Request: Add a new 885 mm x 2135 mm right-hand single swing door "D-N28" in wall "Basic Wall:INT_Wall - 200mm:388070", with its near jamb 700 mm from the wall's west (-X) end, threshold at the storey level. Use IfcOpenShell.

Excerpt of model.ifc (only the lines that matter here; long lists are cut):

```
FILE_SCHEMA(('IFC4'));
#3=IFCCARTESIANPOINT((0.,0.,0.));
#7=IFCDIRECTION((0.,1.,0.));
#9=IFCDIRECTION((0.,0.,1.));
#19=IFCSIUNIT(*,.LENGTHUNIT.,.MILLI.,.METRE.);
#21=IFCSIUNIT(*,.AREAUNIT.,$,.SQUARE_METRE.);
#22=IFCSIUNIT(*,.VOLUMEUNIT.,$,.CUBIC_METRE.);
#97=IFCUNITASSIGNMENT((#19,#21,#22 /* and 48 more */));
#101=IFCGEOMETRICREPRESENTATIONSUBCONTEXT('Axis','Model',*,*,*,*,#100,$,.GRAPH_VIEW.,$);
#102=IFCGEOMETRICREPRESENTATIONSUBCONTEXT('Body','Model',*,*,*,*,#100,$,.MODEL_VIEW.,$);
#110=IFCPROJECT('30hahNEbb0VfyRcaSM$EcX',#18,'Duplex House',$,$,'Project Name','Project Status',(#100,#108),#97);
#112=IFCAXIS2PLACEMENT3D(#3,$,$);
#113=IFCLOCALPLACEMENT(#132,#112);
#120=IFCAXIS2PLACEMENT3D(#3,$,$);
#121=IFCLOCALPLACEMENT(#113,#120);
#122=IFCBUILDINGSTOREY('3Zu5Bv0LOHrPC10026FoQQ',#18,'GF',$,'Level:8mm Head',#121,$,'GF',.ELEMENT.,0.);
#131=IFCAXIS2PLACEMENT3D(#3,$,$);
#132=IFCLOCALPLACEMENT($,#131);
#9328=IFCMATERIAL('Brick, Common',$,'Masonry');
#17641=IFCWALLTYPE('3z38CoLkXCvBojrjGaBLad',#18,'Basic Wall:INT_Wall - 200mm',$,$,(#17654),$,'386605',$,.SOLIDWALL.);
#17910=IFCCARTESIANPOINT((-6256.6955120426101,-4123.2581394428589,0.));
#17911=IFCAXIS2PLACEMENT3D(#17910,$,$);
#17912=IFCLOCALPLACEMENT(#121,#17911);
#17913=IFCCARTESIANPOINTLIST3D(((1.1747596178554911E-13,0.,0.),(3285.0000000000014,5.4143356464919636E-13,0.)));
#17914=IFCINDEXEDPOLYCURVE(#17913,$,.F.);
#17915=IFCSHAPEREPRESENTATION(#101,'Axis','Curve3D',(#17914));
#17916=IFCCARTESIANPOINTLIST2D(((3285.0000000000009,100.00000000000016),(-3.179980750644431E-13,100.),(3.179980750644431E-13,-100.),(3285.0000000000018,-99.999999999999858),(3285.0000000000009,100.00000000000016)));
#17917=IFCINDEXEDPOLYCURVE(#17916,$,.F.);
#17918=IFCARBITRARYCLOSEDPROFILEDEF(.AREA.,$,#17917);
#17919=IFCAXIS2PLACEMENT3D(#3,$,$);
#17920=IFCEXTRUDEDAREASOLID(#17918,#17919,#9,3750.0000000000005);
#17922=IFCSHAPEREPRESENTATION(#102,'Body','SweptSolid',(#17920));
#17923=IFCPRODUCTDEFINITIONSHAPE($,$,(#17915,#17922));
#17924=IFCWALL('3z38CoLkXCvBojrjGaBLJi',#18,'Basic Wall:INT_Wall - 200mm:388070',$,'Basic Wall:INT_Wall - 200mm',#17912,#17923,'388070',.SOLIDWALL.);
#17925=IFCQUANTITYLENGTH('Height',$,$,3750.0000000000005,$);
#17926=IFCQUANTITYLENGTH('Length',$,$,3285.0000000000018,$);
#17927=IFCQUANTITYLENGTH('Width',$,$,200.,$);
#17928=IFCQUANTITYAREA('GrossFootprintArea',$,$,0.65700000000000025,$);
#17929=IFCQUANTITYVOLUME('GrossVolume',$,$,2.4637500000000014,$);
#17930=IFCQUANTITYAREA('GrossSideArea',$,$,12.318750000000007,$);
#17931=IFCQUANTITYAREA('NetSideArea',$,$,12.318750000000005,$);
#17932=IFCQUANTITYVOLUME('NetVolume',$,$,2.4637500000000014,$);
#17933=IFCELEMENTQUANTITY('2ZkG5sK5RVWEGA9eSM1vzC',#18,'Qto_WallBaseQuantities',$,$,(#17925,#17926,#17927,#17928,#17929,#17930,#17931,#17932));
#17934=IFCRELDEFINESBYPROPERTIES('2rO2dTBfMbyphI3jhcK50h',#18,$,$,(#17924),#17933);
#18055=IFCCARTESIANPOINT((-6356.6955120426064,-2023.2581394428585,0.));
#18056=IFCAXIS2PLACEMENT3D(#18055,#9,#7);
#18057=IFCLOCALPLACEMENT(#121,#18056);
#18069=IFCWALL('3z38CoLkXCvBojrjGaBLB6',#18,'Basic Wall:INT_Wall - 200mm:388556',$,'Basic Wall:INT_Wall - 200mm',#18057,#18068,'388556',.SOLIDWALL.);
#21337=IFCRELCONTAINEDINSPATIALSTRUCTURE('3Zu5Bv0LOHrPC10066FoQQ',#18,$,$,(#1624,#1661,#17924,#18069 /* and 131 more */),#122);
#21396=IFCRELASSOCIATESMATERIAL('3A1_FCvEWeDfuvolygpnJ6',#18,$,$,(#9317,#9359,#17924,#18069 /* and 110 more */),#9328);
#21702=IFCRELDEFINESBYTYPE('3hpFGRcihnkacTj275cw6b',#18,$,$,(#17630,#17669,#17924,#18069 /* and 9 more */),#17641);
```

```python
import numpy as np
import ifcopenshell
import ifcopenshell.api.feature
import ifcopenshell.api.geometry
import ifcopenshell.api.pset
import ifcopenshell.api.root
import ifcopenshell.api.spatial
import ifcopenshell.geom
import ifcopenshell.util.element
import ifcopenshell.util.placement
import ifcopenshell.util.representation
import ifcopenshell.util.shape
import ifcopenshell.util.unit

model = ifcopenshell.open("model.ifc")
unit_scale = ifcopenshell.util.unit.calculate_unit_scale(model)
area_scale = ifcopenshell.util.unit.calculate_unit_scale(model, "AREAUNIT")
volume_scale = ifcopenshell.util.unit.calculate_unit_scale(model, "VOLUMEUNIT")
settings = ifcopenshell.geom.settings()


def volume(element):
    """Net volume in cubic metres, openings subtracted."""
    shape = ifcopenshell.geom.create_shape(settings, element)
    return ifcopenshell.util.shape.get_volume(shape.geometry)


wall = model.by_guid("3z38CoLkXCvBojrjGaBLJi")
storey = ifcopenshell.util.element.get_container(wall, ifc_class="IfcBuildingStorey")
context = ifcopenshell.util.representation.get_context(model, "Model", "Body", "MODEL_VIEW")
before = volume(wall)

width, height, from_end, sill = 0.885, 2.135, 0.7, 0.0  # metres

# The wall runs along its own X axis, and the end named is its -X end.
wall_shape = ifcopenshell.geom.create_shape(settings, wall)
x, y, z = ifcopenshell.util.shape.get_vertices(wall_shape.geometry).T
start = x.min() + from_end
face, thickness = float(y.min()), float(y.max() - y.min())
wall_matrix = ifcopenshell.util.placement.get_local_placement(wall.ObjectPlacement)
level = ifcopenshell.util.placement.get_local_placement(storey.ObjectPlacement)[2, 3]


def in_wall(x, y):
    """Placement at x, y metres in the wall's axes, at sill height."""
    matrix = wall_matrix.copy()
    matrix[:, 3] = wall_matrix @ np.array([x / unit_scale, y / unit_scale, 0.0, 1.0])
    matrix[2, 3] = level + sill / unit_scale
    return matrix


# Opening: a box that overshoots both wall faces by 50 mm.
opening = ifcopenshell.api.root.create_entity(model, ifc_class="IfcOpeningElement", predefined_type="OPENING")
box = ifcopenshell.api.geometry.add_wall_representation(
    model, context=context, length=width, height=height, thickness=thickness + 0.1
)
ifcopenshell.api.geometry.assign_representation(model, product=opening, representation=box)
ifcopenshell.api.geometry.edit_object_placement(model, product=opening, matrix=in_wall(start, face - 0.05), is_si=False)
ifcopenshell.api.feature.add_feature(model, feature=opening, element=wall)

door = ifcopenshell.api.root.create_entity(model, ifc_class="IfcDoor", name="D-N28", predefined_type="DOOR")
door.OverallWidth, door.OverallHeight = width / unit_scale, height / unit_scale
door.OperationType = "SINGLE_SWING_RIGHT"
body = ifcopenshell.api.geometry.add_door_representation(
    model,
    context=context,
    overall_width=door.OverallWidth,
    overall_height=door.OverallHeight,
    operation_type="SINGLE_SWING_RIGHT",
    lining_properties={"LiningDepth": thickness / unit_scale, "ThresholdDepth": thickness / unit_scale},
)
ifcopenshell.api.geometry.assign_representation(model, product=door, representation=body)
ifcopenshell.api.spatial.assign_container(model, products=[door], relating_structure=storey)
ifcopenshell.api.feature.add_filling(model, opening=opening, element=door)

# The lining spans the wall, so the door starts at the wall face.
ifcopenshell.api.geometry.edit_object_placement(model, product=door, matrix=in_wall(start, face), is_si=False)

after = volume(wall)

# Update the wall's stored quantities.
qto = model.by_id(ifcopenshell.util.element.get_pset(wall, "Qto_WallBaseQuantities", should_inherit=False)["id"])
ifcopenshell.api.pset.edit_qto(model, qto=qto, properties={
    "NetSideArea": after / thickness / area_scale,
    "NetVolume": after / volume_scale,
})

print(f"wall volume {before:.3f} -> {after:.3f} m3")

model.write("model-out.ifc")
```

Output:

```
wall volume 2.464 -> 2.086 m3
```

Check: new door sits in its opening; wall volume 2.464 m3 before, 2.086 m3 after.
